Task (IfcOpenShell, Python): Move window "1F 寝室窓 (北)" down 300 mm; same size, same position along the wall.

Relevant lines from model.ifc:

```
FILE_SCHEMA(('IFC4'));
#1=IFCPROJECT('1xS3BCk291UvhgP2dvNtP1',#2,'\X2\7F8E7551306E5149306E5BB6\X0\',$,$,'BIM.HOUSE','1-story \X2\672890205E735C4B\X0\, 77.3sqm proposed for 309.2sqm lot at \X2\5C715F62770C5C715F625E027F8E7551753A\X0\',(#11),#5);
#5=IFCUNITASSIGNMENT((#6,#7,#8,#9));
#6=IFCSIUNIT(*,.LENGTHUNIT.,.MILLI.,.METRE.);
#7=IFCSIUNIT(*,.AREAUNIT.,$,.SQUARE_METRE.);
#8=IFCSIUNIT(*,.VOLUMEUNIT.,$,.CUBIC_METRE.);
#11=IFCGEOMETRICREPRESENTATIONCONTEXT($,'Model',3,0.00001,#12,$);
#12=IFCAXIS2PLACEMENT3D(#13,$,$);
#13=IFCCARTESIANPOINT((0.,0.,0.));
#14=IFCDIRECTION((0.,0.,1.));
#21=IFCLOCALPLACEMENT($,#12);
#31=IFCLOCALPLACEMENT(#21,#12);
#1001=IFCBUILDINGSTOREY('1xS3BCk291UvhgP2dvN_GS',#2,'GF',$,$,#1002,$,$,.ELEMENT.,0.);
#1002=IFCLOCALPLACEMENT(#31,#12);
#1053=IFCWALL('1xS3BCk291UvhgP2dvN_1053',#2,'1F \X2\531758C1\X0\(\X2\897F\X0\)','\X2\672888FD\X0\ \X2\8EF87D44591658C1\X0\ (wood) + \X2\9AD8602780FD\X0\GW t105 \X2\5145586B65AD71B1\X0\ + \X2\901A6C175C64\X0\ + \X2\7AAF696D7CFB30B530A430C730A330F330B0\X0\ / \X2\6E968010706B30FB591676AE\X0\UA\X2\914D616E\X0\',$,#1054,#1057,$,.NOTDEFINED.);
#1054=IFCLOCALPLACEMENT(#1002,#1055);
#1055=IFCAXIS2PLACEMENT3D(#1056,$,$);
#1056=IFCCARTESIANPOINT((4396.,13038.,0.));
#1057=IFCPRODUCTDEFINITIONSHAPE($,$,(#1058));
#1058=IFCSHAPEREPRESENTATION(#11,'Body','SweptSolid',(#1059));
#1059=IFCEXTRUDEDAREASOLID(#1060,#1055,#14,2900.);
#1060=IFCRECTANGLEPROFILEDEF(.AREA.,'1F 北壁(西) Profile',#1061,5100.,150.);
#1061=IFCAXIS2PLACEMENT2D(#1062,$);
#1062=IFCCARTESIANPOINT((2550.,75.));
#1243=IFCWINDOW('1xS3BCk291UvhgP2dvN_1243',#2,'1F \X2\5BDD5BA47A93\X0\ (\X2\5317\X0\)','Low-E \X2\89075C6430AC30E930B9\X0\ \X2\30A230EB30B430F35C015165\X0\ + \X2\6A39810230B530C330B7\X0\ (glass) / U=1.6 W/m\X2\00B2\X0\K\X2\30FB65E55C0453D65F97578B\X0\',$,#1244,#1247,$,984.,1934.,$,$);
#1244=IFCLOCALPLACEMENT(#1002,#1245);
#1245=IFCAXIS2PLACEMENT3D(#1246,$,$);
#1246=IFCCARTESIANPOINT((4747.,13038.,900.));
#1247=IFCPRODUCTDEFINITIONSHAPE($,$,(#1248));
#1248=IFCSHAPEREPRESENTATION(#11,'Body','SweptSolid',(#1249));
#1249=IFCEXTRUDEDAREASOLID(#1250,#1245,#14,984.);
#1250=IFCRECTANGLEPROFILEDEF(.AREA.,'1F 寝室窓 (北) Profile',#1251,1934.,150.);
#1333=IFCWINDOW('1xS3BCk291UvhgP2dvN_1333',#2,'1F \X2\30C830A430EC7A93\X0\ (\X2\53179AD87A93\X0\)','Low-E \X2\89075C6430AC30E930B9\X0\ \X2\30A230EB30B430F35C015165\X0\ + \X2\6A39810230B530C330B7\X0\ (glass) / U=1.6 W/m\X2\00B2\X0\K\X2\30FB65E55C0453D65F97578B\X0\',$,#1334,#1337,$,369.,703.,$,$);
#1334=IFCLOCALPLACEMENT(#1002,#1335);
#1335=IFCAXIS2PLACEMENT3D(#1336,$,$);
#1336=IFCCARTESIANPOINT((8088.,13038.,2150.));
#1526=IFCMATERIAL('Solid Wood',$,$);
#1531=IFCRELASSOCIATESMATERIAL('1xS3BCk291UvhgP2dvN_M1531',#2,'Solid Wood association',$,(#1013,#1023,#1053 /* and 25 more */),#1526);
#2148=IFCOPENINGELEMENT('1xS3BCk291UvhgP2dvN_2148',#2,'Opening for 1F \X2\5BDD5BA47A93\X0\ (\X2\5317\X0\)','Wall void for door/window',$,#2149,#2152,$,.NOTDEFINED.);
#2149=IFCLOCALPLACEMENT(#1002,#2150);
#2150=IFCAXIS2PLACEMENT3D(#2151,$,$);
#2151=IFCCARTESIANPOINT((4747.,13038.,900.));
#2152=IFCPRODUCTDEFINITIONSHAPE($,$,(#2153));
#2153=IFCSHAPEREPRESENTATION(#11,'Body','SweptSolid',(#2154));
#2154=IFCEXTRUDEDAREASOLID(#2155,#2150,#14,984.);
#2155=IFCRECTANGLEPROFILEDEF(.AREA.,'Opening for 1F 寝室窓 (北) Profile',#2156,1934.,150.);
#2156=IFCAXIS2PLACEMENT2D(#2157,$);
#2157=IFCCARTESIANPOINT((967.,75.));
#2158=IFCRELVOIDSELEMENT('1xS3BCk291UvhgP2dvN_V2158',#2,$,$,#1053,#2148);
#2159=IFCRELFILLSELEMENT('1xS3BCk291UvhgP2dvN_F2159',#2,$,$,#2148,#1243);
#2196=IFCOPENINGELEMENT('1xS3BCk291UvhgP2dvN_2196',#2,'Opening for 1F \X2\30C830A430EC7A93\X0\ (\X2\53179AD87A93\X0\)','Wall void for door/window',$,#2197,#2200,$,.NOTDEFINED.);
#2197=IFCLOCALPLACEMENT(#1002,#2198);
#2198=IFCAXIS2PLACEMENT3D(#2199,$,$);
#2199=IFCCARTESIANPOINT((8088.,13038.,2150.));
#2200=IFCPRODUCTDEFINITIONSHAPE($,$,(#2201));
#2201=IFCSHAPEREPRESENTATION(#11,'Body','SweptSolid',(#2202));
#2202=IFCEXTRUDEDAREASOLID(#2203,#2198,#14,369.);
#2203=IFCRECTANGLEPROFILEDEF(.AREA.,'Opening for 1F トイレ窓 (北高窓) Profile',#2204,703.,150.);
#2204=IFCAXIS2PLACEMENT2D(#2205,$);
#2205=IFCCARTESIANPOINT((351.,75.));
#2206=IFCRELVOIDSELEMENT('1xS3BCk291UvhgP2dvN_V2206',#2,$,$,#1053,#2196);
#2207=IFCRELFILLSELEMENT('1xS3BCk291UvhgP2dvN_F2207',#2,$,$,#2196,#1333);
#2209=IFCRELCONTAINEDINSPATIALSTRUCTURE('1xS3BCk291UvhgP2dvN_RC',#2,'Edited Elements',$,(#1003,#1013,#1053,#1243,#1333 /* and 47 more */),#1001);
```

```python
import numpy as np
import ifcopenshell
import ifcopenshell.api.geometry
import ifcopenshell.util.placement
import ifcopenshell.util.unit

model = ifcopenshell.open("model.ifc")
unit_scale = ifcopenshell.util.unit.calculate_unit_scale(model)

window = model.by_guid("1xS3BCk291UvhgP2dvN_1243")
opening = window.FillsVoids[0].RelatingOpeningElement
dz = -300.0

shift = np.array([0.0, 0.0, dz])
# The window is not placed relative to its opening, so move both.
for product in (opening, window):
    matrix = ifcopenshell.util.placement.get_local_placement(product.ObjectPlacement)
    matrix[:3, 3] += shift
    ifcopenshell.api.geometry.edit_object_placement(model, product=product, matrix=matrix, is_si=False)

print(f"moved by {dz * unit_scale:+.3f} m")

model.write("model_rev.ifc")
```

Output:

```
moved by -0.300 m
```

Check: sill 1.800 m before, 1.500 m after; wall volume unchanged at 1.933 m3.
